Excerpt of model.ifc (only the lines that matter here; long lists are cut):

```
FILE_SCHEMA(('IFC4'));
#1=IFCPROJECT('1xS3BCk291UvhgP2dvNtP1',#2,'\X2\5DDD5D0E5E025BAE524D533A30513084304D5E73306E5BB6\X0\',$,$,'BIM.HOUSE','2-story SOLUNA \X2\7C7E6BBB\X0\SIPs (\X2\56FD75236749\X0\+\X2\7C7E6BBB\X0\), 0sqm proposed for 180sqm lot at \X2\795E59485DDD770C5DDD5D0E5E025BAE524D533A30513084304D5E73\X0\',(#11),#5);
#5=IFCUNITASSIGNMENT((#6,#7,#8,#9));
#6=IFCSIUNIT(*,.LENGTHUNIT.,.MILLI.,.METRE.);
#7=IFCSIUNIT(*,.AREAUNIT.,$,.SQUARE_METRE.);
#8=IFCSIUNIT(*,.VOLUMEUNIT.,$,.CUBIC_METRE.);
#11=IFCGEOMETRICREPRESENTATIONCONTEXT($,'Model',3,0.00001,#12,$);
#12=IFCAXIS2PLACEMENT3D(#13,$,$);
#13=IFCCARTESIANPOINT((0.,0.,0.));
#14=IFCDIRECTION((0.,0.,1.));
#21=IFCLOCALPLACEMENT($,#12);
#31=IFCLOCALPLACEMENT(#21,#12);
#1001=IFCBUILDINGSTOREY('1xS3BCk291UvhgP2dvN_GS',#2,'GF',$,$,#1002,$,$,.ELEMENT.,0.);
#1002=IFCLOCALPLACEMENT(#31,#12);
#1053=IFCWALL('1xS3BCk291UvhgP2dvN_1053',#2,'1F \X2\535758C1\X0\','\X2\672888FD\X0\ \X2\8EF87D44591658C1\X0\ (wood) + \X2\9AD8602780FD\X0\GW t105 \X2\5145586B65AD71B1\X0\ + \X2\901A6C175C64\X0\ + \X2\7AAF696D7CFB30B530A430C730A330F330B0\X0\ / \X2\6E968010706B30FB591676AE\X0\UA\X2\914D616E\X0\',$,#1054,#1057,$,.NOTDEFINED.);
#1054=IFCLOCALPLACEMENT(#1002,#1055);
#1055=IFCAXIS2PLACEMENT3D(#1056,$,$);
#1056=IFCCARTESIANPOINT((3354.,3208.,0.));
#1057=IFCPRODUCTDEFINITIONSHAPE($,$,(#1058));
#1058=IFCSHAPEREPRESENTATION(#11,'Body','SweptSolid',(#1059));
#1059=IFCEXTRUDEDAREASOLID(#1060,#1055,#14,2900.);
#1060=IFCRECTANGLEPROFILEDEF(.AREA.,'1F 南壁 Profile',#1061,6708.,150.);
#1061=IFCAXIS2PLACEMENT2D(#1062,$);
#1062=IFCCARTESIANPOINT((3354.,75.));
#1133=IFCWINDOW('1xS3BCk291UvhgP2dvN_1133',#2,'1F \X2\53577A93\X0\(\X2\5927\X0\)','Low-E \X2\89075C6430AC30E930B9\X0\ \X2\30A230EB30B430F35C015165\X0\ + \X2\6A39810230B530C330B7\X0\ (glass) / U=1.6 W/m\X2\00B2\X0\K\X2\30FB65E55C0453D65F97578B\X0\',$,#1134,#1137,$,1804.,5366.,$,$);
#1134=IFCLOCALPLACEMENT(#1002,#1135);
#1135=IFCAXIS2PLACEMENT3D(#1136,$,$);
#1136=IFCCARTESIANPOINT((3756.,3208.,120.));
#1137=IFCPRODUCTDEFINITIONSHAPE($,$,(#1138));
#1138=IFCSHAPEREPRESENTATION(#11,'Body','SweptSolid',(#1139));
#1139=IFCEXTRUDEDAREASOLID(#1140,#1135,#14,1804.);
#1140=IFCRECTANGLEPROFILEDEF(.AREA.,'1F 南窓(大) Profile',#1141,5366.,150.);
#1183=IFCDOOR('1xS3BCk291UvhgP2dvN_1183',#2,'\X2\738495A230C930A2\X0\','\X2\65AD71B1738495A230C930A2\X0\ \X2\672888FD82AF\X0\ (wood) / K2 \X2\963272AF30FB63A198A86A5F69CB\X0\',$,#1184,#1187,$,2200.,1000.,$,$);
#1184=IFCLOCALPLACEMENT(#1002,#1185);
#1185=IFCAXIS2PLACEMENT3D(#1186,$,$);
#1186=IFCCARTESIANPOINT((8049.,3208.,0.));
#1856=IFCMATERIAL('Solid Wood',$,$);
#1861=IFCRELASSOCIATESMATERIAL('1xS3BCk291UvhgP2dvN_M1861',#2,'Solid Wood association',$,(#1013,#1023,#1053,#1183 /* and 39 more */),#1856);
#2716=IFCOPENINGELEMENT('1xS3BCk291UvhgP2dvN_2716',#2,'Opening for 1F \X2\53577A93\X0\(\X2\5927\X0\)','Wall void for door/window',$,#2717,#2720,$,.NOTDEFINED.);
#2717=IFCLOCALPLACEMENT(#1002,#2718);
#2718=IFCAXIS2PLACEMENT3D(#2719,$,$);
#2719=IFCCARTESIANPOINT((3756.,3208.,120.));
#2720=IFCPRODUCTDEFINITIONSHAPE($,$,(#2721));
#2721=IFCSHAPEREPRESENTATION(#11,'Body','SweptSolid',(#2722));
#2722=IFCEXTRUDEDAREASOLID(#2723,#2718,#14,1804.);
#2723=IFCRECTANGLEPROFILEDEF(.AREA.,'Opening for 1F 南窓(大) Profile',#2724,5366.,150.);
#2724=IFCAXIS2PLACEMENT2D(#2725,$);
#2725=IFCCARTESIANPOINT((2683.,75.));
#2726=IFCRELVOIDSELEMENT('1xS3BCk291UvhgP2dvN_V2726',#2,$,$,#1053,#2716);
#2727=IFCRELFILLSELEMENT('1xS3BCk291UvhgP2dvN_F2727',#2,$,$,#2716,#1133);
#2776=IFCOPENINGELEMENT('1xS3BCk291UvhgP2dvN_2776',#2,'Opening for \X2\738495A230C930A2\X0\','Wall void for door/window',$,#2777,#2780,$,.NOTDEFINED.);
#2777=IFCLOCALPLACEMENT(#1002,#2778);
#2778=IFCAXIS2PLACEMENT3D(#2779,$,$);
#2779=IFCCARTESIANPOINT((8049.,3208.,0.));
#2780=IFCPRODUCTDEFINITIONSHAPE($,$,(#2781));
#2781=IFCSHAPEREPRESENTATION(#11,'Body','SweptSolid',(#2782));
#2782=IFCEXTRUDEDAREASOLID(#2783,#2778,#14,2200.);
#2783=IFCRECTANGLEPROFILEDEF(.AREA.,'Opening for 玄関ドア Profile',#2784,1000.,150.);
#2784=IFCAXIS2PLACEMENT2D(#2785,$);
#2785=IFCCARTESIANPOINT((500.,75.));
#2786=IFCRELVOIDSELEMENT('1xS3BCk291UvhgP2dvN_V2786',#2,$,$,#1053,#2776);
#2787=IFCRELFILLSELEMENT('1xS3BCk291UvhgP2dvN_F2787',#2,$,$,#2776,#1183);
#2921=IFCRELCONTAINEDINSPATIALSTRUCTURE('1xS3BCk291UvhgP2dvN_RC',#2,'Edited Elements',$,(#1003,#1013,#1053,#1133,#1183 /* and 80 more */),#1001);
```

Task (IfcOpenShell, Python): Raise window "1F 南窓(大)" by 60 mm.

```python
import numpy as np
import ifcopenshell
import ifcopenshell.api.geometry
import ifcopenshell.util.placement
import ifcopenshell.util.unit

model = ifcopenshell.open("model.ifc")
unit_scale = ifcopenshell.util.unit.calculate_unit_scale(model)

window = model.by_id(1133)
opening = window.FillsVoids[0].RelatingOpeningElement
dz = 60.0

shift = np.array([0.0, 0.0, dz])
# The window is not placed relative to its opening, so move both.
for product in (opening, window):
    matrix = ifcopenshell.util.placement.get_local_placement(product.ObjectPlacement)
    matrix[:3, 3] += shift
    ifcopenshell.api.geometry.edit_object_placement(model, product=product, matrix=matrix, is_si=False)

print(f"moved by {dz * unit_scale:+.3f} m")

model.write("model_edited.ifc")
```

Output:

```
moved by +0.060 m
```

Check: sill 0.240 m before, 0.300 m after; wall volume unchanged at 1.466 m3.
